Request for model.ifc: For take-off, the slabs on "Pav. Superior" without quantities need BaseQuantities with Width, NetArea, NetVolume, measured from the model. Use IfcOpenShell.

First a look at what the model holds.

```python
import ifcopenshell
import ifcopenshell.util.element
import ifcopenshell.util.unit

model = ifcopenshell.open("model.ifc")
print(model.schema)
for unit_type in ("LENGTHUNIT", "AREAUNIT", "VOLUMEUNIT"):
    print(unit_type, ifcopenshell.util.unit.calculate_unit_scale(model, unit_type))
storey = next(s for s in model.by_type("IfcBuildingStorey") if s.Name == "Pav. Superior")
slabs = [e for e in ifcopenshell.util.element.get_decomposition(storey) if e.is_a("IfcSlab")]
for e in sorted(slabs, key=lambda e: e.id()):
    print(e.id(), e.is_a(), e.Name, list(ifcopenshell.util.element.get_psets(e, qtos_only=True)), sep=" | ")
```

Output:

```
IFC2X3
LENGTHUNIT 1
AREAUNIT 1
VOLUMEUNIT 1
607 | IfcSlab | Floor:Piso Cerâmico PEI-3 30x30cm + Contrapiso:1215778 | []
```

```python
import ifcopenshell
import ifcopenshell.api.pset
import ifcopenshell.geom
import ifcopenshell.util.element
import ifcopenshell.util.shape
import ifcopenshell.util.unit

model = ifcopenshell.open("model.ifc")
unit_scale = ifcopenshell.util.unit.calculate_unit_scale(model)
area_scale = ifcopenshell.util.unit.calculate_unit_scale(model, "AREAUNIT")
volume_scale = ifcopenshell.util.unit.calculate_unit_scale(model, "VOLUMEUNIT")
settings = ifcopenshell.geom.settings()

storey = next(s for s in model.by_type("IfcBuildingStorey") if s.Name == "Pav. Superior")
slabs = [e for e in ifcopenshell.util.element.get_decomposition(storey) if e.is_a("IfcSlab")]

for e in sorted(slabs, key=lambda e: e.id()):
    if ifcopenshell.util.element.get_psets(e, qtos_only=True, should_inherit=False):
        continue
    # Geometry comes back in metres, in the element's own axes.
    shape = ifcopenshell.geom.create_shape(settings, e)
    values = {
        "Width": ifcopenshell.util.shape.get_z(shape.geometry) / unit_scale,
        "NetArea": ifcopenshell.util.shape.get_footprint_area(shape.geometry) / area_scale,
        "NetVolume": ifcopenshell.util.shape.get_volume(shape.geometry) / volume_scale,
    }
    qto = ifcopenshell.api.pset.add_qto(model, product=e, name="BaseQuantities")
    ifcopenshell.api.pset.edit_qto(model, qto=qto, properties=values)
    print(e.id(), {k: round(v, 3) for k, v in values.items()})

model.write("model_rev.ifc")
```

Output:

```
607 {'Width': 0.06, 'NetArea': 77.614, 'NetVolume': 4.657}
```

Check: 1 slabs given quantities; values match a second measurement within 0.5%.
